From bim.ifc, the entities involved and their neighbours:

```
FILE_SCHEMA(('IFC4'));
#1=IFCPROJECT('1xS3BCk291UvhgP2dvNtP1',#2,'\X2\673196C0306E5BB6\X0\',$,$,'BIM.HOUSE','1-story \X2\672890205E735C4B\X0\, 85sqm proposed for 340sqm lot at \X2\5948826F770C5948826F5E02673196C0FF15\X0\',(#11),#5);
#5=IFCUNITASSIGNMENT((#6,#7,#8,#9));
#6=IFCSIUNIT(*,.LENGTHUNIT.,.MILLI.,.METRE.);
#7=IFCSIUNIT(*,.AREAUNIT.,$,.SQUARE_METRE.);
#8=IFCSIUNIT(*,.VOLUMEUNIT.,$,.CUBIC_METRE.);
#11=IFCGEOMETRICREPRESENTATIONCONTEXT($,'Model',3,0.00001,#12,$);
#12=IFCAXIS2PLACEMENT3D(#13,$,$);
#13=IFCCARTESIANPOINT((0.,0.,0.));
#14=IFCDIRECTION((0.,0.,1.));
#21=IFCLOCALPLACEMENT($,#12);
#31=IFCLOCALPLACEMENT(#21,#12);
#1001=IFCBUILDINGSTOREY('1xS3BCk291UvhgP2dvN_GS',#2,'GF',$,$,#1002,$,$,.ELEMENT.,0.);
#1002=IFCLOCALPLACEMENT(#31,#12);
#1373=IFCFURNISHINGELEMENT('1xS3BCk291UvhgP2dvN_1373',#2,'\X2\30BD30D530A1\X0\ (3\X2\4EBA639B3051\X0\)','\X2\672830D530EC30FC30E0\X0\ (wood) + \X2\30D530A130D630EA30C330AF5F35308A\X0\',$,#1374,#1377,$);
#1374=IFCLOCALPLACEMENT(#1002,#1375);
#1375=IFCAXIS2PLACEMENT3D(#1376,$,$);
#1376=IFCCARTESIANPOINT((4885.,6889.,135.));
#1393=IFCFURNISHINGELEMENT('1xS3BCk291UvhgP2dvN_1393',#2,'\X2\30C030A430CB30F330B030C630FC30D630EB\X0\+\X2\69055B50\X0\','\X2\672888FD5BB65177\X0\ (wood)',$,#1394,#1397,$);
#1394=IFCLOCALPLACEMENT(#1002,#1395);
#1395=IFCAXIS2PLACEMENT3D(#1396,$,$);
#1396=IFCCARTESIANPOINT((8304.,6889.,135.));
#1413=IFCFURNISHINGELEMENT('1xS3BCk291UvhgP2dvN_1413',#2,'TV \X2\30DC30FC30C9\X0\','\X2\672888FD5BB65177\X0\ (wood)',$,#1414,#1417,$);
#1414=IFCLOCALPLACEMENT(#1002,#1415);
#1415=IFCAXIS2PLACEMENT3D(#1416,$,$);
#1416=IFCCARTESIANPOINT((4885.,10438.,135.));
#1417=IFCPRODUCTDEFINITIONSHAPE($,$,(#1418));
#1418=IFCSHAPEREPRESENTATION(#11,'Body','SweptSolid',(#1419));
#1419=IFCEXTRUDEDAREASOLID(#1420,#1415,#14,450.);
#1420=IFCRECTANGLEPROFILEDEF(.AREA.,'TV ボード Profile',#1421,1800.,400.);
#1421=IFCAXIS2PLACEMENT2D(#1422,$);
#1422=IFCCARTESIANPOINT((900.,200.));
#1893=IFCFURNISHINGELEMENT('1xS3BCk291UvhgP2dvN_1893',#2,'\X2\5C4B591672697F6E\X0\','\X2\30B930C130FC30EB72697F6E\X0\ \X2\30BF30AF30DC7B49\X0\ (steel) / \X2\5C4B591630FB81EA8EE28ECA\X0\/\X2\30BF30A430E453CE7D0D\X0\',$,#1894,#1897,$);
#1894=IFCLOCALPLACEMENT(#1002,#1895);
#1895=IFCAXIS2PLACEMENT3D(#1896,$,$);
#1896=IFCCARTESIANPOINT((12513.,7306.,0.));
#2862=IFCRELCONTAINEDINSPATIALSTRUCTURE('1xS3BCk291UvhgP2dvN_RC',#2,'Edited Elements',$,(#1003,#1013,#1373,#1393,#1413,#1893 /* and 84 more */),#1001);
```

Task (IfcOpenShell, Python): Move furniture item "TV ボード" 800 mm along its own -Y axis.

```python
import ifcopenshell
import ifcopenshell.api.geometry
import ifcopenshell.util.placement

model = ifcopenshell.open("bim.ifc")

item = model.by_guid("1xS3BCk291UvhgP2dvN_1413")
matrix = ifcopenshell.util.placement.get_local_placement(item.ObjectPlacement)
matrix[:3, 3] -= matrix[:3, 1] * 800.0
ifcopenshell.api.geometry.edit_object_placement(model, product=item, matrix=matrix, is_si=False)

print(ifcopenshell.util.placement.get_local_placement(item.ObjectPlacement).round(3) + 0.0)

model.write("bim_v2.ifc")
```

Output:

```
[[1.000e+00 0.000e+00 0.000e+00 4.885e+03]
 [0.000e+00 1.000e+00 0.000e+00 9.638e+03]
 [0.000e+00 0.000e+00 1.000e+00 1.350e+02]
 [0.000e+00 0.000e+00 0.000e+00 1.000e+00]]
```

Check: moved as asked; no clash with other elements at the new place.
